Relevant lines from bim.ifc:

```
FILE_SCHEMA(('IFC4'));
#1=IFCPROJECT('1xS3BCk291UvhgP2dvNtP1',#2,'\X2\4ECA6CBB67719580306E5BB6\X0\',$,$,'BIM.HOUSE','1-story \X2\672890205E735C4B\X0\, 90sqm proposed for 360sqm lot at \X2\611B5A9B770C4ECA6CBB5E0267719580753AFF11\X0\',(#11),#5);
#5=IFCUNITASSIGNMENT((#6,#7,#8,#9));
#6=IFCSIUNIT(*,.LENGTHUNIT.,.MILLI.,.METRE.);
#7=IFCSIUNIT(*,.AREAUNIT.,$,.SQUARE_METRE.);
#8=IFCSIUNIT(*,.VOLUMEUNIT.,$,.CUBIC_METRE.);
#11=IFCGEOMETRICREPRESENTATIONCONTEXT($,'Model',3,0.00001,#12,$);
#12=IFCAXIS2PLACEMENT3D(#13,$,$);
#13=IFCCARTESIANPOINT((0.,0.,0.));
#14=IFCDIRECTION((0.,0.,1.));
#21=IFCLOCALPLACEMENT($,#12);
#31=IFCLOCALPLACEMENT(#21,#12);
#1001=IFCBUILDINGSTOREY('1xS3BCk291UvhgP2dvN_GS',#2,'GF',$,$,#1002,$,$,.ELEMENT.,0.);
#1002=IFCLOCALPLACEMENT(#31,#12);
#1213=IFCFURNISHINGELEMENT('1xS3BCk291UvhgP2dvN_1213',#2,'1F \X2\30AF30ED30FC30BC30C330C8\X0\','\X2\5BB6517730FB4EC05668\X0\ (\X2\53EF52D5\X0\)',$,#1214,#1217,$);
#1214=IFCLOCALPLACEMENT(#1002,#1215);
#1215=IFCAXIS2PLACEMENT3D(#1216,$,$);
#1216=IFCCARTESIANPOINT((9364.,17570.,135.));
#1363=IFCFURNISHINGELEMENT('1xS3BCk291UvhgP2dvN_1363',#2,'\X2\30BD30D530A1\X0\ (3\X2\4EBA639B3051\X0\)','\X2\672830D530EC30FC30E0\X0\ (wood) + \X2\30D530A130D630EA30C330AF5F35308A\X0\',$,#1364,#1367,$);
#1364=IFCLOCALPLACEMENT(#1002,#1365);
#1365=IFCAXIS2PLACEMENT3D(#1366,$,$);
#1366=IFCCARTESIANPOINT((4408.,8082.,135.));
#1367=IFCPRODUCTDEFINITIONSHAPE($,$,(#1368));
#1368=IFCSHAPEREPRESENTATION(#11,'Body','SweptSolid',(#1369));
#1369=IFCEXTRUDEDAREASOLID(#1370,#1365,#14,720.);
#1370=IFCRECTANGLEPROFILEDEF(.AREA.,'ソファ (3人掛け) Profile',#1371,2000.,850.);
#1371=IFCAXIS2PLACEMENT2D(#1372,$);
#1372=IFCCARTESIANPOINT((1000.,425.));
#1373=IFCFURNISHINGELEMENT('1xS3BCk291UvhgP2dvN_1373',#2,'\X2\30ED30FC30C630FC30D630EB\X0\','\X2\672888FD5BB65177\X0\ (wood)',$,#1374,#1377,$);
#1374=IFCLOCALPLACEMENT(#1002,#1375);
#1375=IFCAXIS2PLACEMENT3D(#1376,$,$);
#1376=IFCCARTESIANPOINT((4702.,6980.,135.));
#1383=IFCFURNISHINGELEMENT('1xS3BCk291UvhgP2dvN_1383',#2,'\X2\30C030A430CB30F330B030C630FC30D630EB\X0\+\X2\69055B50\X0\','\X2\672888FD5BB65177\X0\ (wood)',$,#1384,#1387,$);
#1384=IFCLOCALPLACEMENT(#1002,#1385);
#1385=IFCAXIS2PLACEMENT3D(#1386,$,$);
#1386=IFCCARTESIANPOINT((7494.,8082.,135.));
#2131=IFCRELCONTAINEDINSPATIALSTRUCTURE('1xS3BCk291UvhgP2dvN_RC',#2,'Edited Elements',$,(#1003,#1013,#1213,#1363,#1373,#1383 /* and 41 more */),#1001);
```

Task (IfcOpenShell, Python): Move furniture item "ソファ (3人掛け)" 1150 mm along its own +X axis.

```python
import ifcopenshell
import ifcopenshell.api.geometry
import ifcopenshell.util.placement

model = ifcopenshell.open("bim.ifc")

item = model.by_guid("1xS3BCk291UvhgP2dvN_1363")
matrix = ifcopenshell.util.placement.get_local_placement(item.ObjectPlacement)
matrix[:3, 3] += matrix[:3, 0] * 1150.0
ifcopenshell.api.geometry.edit_object_placement(model, product=item, matrix=matrix, is_si=False)

print(ifcopenshell.util.placement.get_local_placement(item.ObjectPlacement).round(3) + 0.0)

model.write("bim_updated.ifc")
```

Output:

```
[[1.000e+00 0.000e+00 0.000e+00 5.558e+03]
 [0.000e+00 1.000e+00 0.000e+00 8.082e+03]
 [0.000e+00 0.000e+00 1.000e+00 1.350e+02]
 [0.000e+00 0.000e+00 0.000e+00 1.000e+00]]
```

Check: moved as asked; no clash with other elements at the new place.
